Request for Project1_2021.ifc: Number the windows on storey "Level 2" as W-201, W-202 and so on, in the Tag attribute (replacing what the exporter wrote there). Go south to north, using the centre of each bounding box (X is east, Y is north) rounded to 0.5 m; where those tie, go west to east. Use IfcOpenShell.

First a look at what the model holds.

```python
import ifcopenshell
import ifcopenshell.util.element
import ifcopenshell.util.placement

model = ifcopenshell.open("Project1_2021.ifc")
print(model.schema)
storey = next(s for s in model.by_type("IfcBuildingStorey") if s.Name == "Level 2")
windows = [e for e in ifcopenshell.util.element.get_decomposition(storey) if e.is_a("IfcWindow")]
for e in sorted(windows, key=lambda e: e.id()):
    origin = ifcopenshell.util.placement.get_local_placement(e.ObjectPlacement)[:3, 3]
    print(e.id(), e.Tag, e.Name, origin.round(2) + 0.0, sep=" | ")
```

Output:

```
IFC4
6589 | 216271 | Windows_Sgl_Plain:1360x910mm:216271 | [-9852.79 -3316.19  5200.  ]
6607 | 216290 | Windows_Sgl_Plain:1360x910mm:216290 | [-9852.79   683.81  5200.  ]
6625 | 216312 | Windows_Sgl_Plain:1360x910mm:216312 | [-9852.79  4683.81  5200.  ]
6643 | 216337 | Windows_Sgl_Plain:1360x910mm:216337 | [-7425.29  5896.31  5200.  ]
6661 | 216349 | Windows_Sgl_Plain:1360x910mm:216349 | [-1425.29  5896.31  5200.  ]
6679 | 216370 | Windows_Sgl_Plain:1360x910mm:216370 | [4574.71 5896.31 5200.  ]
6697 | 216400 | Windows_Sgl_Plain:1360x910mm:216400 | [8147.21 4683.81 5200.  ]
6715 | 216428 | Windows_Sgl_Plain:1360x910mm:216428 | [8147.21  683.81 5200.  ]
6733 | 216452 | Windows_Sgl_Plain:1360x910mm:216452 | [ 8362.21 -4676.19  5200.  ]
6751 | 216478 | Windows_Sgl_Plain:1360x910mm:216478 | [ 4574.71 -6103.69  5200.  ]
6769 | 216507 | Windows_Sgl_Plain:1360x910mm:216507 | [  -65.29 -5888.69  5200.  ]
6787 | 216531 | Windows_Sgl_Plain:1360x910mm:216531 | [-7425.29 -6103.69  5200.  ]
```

```python
import ifcopenshell
import ifcopenshell.geom
import ifcopenshell.util.element
import ifcopenshell.util.shape

model = ifcopenshell.open("Project1_2021.ifc")
settings = ifcopenshell.geom.settings()
settings.set("use-world-coords", True)


def centre(element):
    shape = ifcopenshell.geom.create_shape(settings, element)
    return ifcopenshell.util.shape.get_bbox_centroid(shape.geometry)


storey = next(s for s in model.by_type("IfcBuildingStorey") if s.Name == "Level 2")
windows = [e for e in ifcopenshell.util.element.get_decomposition(storey) if e.is_a("IfcWindow")]

# Insertion points can sit at a corner or the storey origin, so sort by the geometry (in metres).
centres = {e: centre(e) for e in windows}
windows.sort(key=lambda e: (round(centres[e][1] / 0.5), centres[e][0]))

for i, e in enumerate(windows, start=1):
    number = f"W-2{i:02d}"
    e.Tag = number
    print(e.id(), number)

model.write("Project1_2021_v2.ifc")
```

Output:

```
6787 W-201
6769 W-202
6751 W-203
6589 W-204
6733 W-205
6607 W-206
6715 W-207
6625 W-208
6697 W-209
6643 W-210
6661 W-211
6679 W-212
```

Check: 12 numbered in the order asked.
